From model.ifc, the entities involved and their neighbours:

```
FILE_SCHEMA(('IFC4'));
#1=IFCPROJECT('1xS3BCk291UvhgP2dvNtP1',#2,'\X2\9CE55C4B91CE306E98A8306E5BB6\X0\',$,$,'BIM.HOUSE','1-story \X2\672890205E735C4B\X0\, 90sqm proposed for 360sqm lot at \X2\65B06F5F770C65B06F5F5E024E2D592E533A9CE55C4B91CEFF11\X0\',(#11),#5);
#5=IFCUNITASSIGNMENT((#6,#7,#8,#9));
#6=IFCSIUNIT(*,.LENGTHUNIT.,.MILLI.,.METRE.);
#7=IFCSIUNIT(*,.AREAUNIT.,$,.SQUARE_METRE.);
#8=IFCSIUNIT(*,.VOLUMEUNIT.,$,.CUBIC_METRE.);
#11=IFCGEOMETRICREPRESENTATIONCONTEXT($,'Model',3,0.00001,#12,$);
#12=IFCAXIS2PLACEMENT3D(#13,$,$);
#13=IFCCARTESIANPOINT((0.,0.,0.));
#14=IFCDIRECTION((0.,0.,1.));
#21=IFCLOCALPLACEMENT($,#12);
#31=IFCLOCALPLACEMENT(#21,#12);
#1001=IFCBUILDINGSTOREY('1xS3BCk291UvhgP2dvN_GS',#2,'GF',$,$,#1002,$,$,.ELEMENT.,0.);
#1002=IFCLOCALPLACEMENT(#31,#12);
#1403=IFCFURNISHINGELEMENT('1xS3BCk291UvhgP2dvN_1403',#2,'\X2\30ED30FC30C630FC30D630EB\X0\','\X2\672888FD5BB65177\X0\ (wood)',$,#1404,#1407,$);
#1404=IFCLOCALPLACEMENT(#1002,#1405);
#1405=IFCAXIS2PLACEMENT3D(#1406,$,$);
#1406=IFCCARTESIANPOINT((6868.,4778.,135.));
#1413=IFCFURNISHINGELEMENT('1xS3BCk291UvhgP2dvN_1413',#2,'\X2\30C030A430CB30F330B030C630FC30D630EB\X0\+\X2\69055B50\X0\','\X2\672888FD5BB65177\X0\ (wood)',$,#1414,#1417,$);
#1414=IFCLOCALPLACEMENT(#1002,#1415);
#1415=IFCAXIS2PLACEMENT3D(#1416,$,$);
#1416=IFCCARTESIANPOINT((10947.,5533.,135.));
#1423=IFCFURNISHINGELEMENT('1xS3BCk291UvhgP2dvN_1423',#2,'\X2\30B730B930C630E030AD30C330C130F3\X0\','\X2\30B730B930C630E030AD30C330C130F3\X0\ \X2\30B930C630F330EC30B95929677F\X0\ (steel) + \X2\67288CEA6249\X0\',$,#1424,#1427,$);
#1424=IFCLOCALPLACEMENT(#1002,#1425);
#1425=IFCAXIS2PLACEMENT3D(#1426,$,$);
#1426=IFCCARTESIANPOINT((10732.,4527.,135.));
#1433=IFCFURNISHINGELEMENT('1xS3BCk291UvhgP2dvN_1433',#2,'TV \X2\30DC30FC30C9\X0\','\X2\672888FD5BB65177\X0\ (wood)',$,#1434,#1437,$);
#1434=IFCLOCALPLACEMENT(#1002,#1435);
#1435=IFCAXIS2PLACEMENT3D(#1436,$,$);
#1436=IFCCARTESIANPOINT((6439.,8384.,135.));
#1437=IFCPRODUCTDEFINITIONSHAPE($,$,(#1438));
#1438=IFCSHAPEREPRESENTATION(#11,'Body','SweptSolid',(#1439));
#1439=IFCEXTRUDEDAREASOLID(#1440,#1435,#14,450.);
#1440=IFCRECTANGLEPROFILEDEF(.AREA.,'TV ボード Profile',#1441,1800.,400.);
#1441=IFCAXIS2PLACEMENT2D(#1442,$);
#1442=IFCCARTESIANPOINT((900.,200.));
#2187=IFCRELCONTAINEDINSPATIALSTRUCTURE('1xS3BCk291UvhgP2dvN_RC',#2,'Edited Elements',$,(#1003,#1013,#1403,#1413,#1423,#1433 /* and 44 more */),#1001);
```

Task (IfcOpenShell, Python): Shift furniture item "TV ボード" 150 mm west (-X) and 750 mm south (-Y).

```python
import ifcopenshell
import ifcopenshell.api.geometry
import ifcopenshell.util.placement
import ifcopenshell.util.unit

model = ifcopenshell.open("model.ifc")
unit_scale = ifcopenshell.util.unit.calculate_unit_scale(model)

item = model.by_guid("1xS3BCk291UvhgP2dvN_1433")
matrix = ifcopenshell.util.placement.get_local_placement(item.ObjectPlacement)
matrix[0, 3] -= 0.15 / unit_scale
matrix[1, 3] -= 0.75 / unit_scale
ifcopenshell.api.geometry.edit_object_placement(model, product=item, matrix=matrix, is_si=False)

print(ifcopenshell.util.placement.get_local_placement(item.ObjectPlacement).round(3) + 0.0)

model.write("model-out.ifc")
```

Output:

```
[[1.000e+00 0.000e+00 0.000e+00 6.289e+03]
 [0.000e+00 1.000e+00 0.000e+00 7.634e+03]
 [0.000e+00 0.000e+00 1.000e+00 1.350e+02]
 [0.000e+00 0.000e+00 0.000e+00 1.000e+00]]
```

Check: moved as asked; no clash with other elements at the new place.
